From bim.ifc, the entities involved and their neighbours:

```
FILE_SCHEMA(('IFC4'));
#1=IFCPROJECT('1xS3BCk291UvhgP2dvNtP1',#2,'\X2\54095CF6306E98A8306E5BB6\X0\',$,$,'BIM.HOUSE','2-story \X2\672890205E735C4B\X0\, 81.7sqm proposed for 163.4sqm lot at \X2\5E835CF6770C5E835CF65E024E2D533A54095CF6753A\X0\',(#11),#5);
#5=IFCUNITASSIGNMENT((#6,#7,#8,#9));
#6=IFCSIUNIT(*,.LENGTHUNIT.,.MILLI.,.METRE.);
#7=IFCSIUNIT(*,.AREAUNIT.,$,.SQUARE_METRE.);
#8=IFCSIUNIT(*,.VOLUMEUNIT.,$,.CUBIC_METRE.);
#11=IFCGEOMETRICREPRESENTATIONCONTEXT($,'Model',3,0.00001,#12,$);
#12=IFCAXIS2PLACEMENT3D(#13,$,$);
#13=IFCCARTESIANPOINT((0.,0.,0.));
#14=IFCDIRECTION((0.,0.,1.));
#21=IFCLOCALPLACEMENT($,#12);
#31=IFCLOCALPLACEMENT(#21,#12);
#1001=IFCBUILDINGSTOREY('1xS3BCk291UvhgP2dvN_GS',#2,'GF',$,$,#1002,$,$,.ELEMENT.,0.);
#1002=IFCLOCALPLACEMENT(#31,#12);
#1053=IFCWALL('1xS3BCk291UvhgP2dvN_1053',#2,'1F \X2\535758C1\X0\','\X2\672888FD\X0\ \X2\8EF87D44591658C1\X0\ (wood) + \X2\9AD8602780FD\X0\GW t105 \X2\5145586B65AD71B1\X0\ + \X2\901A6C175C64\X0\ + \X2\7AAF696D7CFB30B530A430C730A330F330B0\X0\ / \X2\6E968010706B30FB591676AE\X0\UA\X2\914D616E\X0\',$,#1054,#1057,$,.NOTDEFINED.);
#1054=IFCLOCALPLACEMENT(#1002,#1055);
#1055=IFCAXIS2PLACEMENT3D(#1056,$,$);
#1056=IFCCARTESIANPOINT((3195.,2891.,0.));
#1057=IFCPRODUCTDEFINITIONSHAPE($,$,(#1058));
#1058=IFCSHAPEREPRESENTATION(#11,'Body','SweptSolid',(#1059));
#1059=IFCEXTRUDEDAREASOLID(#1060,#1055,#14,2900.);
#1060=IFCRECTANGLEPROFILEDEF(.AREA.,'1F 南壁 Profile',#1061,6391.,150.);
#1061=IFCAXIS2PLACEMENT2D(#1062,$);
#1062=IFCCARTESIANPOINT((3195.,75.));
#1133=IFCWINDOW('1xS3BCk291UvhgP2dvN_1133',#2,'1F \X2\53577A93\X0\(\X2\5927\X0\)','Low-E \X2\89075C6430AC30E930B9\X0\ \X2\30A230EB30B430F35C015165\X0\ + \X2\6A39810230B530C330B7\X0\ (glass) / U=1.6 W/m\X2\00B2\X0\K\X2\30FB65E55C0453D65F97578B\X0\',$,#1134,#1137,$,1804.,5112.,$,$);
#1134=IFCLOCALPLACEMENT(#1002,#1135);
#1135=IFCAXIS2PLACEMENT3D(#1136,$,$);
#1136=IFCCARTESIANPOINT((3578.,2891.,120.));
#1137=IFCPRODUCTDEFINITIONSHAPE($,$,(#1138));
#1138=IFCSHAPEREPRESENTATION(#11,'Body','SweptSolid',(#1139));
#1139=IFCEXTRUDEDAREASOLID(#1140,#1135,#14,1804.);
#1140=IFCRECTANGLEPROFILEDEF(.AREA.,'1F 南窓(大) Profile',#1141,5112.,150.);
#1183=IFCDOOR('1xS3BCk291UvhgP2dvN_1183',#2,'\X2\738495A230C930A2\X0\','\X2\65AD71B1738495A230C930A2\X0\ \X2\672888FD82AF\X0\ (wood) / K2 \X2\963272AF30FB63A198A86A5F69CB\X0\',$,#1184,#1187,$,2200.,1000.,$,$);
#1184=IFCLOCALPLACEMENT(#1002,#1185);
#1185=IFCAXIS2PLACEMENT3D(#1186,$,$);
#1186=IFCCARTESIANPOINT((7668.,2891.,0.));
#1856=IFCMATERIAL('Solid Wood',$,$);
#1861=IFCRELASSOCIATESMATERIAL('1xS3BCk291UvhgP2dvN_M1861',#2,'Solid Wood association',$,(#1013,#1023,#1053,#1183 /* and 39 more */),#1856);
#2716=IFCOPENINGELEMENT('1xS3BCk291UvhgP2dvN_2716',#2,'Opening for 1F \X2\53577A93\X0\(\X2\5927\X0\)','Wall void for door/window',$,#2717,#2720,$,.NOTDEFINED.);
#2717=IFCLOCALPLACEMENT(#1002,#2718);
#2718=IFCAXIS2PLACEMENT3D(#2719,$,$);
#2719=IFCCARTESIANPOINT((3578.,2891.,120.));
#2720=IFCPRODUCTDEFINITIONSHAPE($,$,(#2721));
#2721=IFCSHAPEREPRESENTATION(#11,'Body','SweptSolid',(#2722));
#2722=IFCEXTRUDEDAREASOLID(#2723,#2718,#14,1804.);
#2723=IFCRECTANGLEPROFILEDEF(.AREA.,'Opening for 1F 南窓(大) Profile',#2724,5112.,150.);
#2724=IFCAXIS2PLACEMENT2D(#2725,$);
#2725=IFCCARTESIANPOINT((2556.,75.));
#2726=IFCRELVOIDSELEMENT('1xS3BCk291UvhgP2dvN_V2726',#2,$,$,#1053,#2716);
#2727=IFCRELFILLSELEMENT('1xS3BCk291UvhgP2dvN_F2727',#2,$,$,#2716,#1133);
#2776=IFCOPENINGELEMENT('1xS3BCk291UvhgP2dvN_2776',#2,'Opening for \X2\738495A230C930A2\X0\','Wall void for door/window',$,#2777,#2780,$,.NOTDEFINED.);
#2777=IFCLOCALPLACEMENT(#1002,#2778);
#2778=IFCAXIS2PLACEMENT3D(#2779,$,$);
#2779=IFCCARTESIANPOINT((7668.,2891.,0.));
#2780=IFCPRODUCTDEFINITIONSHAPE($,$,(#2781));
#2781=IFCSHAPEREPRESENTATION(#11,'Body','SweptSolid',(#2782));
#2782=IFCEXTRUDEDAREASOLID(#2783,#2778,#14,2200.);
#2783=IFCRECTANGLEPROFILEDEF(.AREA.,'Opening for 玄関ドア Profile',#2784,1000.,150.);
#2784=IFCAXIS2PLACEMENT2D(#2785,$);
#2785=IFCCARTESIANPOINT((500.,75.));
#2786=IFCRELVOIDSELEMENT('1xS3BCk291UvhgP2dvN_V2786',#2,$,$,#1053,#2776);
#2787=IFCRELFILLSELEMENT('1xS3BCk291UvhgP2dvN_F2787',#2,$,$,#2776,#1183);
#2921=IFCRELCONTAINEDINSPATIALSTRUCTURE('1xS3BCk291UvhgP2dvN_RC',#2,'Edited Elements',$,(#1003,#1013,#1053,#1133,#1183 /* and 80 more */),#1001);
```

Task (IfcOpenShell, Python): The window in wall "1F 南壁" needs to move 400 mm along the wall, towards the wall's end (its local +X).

```python
import ifcopenshell
import ifcopenshell.api.geometry
import ifcopenshell.util.placement
import ifcopenshell.util.unit

model = ifcopenshell.open("bim.ifc")
unit_scale = ifcopenshell.util.unit.calculate_unit_scale(model)

window = model.by_guid("1xS3BCk291UvhgP2dvN_1133")
opening = window.FillsVoids[0].RelatingOpeningElement
wall = opening.VoidsElements[0].RelatingBuildingElement

wall_matrix = ifcopenshell.util.placement.get_local_placement(wall.ObjectPlacement)
shift = wall_matrix[:3, 0] * 0.4 / unit_scale
before = ifcopenshell.util.placement.get_local_placement(window.ObjectPlacement)[:3, 3].copy()

# The window is not placed relative to its opening, so move both.
for product in (opening, window):
    matrix = ifcopenshell.util.placement.get_local_placement(product.ObjectPlacement)
    matrix[:3, 3] += shift
    ifcopenshell.api.geometry.edit_object_placement(model, product=product, matrix=matrix, is_si=False)

after = ifcopenshell.util.placement.get_local_placement(window.ObjectPlacement)[:3, 3]
print("window moved by", (after - before).round(3) + 0.0)

model.write("bim-out.ifc")
```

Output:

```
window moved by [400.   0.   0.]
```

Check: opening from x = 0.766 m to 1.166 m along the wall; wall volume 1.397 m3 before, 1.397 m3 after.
